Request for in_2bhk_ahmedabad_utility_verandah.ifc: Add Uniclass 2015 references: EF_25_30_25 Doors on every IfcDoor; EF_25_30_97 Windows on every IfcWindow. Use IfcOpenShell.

First a look at what the model holds.

```python
import ifcopenshell

model = ifcopenshell.open("in_2bhk_ahmedabad_utility_verandah.ifc")
print(model.schema)
print("classifications:", [c.Name for c in model.by_type("IfcClassification")])
for ifc_class in ("IfcDoor", "IfcRoof", "IfcStair", "IfcWall", "IfcWindow"):
    print(ifc_class, len(model.by_type(ifc_class)))
```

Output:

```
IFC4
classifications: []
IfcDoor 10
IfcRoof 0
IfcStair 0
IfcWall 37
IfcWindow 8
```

```python
import ifcopenshell
import ifcopenshell.api.classification

model = ifcopenshell.open("in_2bhk_ahmedabad_utility_verandah.ifc")

system = ifcopenshell.api.classification.add_classification(model, classification="Uniclass 2015")

codes = {
    "IfcDoor": ("EF_25_30_25", "Doors"),
    "IfcWindow": ("EF_25_30_97", "Windows"),
}
for ifc_class, (code, name) in codes.items():
    products = model.by_type(ifc_class)
    ifcopenshell.api.classification.add_reference(
        model, products=products, classification=system, identification=code, name=name
    )
    print(code, len(products))

model.write("in_2bhk_ahmedabad_utility_verandah_rev.ifc")
```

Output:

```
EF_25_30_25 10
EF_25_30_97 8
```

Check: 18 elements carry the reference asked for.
